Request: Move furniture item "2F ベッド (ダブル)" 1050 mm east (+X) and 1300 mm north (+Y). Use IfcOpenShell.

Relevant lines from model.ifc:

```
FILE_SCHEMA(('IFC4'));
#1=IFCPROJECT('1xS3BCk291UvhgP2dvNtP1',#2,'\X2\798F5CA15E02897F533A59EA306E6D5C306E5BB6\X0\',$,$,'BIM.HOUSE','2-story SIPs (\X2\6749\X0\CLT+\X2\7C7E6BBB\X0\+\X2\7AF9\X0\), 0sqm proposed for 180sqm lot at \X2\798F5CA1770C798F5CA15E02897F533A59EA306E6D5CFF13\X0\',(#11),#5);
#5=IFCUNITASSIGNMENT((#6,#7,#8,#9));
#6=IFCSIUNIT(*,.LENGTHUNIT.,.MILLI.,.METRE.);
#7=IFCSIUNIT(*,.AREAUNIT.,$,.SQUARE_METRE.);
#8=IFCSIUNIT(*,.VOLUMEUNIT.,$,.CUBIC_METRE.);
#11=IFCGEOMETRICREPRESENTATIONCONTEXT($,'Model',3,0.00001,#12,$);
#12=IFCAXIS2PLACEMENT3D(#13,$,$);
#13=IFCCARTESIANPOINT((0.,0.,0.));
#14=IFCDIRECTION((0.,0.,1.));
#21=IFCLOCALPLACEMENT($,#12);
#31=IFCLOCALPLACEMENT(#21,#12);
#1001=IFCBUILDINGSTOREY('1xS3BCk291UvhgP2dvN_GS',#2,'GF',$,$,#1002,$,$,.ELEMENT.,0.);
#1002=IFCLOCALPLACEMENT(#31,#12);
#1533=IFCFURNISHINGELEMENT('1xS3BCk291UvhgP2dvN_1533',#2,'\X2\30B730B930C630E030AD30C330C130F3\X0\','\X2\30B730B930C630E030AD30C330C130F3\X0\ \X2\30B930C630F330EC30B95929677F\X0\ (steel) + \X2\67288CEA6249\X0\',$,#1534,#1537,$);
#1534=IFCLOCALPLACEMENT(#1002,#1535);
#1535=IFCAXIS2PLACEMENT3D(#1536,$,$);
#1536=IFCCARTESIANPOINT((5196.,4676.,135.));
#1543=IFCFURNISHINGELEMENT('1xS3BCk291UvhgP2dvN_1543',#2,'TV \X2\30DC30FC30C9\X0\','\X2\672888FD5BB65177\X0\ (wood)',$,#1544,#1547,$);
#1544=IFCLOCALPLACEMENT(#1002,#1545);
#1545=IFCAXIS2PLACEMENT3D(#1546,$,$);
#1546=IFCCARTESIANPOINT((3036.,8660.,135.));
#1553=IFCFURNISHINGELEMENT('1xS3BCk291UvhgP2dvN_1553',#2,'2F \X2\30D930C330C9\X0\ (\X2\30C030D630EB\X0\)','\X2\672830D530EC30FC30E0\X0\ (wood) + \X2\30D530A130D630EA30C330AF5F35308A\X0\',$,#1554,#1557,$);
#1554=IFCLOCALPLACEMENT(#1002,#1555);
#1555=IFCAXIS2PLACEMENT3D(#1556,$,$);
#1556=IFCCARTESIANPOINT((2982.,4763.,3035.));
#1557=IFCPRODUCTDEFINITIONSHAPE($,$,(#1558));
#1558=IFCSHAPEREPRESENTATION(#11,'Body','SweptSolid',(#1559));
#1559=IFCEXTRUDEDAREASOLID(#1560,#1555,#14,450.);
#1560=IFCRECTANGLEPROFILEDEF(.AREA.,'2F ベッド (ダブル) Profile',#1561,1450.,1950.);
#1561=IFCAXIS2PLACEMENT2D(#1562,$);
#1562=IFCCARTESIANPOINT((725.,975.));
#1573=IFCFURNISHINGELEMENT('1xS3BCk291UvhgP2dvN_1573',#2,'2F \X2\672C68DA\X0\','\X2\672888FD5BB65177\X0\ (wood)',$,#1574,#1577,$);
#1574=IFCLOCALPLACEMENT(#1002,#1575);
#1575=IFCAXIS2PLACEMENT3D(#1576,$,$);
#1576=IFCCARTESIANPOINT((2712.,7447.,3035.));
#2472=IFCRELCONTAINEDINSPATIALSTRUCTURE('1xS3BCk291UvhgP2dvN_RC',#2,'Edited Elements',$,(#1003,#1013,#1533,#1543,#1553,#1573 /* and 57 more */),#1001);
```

```python
import ifcopenshell
import ifcopenshell.api.geometry
import ifcopenshell.util.placement
import ifcopenshell.util.unit

model = ifcopenshell.open("model.ifc")
unit_scale = ifcopenshell.util.unit.calculate_unit_scale(model)

item = model.by_id(1553)
matrix = ifcopenshell.util.placement.get_local_placement(item.ObjectPlacement)
matrix[0, 3] += 1.05 / unit_scale
matrix[1, 3] += 1.3 / unit_scale
ifcopenshell.api.geometry.edit_object_placement(model, product=item, matrix=matrix, is_si=False)

print(ifcopenshell.util.placement.get_local_placement(item.ObjectPlacement).round(3) + 0.0)

model.write("model_edited.ifc")
```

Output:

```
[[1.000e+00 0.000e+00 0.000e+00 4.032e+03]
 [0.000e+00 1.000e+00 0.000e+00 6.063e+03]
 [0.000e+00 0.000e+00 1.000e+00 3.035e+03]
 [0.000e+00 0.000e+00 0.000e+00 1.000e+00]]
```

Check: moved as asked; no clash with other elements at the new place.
